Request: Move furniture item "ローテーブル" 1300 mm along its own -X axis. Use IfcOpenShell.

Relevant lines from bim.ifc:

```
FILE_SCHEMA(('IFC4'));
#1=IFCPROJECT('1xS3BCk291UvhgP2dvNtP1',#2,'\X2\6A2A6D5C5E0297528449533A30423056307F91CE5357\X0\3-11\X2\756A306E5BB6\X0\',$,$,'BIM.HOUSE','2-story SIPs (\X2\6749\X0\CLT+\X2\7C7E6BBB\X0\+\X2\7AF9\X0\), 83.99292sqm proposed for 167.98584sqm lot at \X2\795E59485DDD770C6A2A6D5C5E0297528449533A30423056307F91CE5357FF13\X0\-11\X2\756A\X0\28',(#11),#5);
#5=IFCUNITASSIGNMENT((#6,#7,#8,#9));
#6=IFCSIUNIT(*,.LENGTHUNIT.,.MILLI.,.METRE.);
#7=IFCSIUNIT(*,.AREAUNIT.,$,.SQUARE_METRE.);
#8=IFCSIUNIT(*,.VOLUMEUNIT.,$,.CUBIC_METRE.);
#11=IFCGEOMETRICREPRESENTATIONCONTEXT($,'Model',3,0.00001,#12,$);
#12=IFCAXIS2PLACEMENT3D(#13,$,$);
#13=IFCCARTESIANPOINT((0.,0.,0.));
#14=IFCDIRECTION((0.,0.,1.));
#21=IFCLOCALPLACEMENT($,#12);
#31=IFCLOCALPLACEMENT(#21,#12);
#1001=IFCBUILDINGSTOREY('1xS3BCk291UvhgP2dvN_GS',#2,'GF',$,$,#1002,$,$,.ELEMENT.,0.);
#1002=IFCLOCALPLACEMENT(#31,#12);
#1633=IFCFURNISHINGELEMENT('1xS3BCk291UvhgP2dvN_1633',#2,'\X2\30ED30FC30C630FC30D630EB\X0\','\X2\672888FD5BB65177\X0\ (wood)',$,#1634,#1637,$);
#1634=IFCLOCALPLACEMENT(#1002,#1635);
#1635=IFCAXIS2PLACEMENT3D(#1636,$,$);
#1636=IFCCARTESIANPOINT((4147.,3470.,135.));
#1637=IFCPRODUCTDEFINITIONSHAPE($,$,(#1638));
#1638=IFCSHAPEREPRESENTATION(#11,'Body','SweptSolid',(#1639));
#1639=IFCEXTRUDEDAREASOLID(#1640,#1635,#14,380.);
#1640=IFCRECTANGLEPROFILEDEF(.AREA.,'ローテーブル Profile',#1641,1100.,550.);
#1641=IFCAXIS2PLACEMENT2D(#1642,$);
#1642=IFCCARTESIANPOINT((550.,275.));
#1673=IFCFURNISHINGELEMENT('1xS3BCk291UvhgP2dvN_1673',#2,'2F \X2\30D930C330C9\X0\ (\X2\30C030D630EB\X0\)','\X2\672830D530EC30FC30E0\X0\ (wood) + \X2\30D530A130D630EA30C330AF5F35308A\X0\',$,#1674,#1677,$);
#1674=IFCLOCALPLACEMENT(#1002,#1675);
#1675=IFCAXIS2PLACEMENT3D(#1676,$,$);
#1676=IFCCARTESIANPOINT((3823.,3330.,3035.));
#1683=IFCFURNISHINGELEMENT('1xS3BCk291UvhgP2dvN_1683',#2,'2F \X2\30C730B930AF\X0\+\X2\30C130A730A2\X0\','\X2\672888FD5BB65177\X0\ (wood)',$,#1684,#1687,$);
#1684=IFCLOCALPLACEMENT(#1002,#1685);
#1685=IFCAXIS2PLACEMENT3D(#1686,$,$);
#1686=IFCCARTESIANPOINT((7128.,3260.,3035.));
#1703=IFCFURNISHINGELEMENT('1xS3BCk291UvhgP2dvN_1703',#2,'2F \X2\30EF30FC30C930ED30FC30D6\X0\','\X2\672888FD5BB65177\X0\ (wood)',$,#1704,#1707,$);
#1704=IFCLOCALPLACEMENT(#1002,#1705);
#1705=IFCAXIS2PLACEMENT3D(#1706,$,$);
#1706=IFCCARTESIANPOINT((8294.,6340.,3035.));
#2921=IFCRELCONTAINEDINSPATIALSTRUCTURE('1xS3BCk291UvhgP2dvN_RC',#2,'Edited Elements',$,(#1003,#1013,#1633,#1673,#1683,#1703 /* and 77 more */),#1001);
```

```python
import ifcopenshell
import ifcopenshell.api.geometry
import ifcopenshell.util.placement
import ifcopenshell.util.unit

model = ifcopenshell.open("bim.ifc")
unit_scale = ifcopenshell.util.unit.calculate_unit_scale(model)

item = model.by_guid("1xS3BCk291UvhgP2dvN_1633")
matrix = ifcopenshell.util.placement.get_local_placement(item.ObjectPlacement)
matrix[:3, 3] -= matrix[:3, 0] * 1.3 / unit_scale
ifcopenshell.api.geometry.edit_object_placement(model, product=item, matrix=matrix, is_si=False)

print(ifcopenshell.util.placement.get_local_placement(item.ObjectPlacement).round(3) + 0.0)

model.write("bim_v2.ifc")
```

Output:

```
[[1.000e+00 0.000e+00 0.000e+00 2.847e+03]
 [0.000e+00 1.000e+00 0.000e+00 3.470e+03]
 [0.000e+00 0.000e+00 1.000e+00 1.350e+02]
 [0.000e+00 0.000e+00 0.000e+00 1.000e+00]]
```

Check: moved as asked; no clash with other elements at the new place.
